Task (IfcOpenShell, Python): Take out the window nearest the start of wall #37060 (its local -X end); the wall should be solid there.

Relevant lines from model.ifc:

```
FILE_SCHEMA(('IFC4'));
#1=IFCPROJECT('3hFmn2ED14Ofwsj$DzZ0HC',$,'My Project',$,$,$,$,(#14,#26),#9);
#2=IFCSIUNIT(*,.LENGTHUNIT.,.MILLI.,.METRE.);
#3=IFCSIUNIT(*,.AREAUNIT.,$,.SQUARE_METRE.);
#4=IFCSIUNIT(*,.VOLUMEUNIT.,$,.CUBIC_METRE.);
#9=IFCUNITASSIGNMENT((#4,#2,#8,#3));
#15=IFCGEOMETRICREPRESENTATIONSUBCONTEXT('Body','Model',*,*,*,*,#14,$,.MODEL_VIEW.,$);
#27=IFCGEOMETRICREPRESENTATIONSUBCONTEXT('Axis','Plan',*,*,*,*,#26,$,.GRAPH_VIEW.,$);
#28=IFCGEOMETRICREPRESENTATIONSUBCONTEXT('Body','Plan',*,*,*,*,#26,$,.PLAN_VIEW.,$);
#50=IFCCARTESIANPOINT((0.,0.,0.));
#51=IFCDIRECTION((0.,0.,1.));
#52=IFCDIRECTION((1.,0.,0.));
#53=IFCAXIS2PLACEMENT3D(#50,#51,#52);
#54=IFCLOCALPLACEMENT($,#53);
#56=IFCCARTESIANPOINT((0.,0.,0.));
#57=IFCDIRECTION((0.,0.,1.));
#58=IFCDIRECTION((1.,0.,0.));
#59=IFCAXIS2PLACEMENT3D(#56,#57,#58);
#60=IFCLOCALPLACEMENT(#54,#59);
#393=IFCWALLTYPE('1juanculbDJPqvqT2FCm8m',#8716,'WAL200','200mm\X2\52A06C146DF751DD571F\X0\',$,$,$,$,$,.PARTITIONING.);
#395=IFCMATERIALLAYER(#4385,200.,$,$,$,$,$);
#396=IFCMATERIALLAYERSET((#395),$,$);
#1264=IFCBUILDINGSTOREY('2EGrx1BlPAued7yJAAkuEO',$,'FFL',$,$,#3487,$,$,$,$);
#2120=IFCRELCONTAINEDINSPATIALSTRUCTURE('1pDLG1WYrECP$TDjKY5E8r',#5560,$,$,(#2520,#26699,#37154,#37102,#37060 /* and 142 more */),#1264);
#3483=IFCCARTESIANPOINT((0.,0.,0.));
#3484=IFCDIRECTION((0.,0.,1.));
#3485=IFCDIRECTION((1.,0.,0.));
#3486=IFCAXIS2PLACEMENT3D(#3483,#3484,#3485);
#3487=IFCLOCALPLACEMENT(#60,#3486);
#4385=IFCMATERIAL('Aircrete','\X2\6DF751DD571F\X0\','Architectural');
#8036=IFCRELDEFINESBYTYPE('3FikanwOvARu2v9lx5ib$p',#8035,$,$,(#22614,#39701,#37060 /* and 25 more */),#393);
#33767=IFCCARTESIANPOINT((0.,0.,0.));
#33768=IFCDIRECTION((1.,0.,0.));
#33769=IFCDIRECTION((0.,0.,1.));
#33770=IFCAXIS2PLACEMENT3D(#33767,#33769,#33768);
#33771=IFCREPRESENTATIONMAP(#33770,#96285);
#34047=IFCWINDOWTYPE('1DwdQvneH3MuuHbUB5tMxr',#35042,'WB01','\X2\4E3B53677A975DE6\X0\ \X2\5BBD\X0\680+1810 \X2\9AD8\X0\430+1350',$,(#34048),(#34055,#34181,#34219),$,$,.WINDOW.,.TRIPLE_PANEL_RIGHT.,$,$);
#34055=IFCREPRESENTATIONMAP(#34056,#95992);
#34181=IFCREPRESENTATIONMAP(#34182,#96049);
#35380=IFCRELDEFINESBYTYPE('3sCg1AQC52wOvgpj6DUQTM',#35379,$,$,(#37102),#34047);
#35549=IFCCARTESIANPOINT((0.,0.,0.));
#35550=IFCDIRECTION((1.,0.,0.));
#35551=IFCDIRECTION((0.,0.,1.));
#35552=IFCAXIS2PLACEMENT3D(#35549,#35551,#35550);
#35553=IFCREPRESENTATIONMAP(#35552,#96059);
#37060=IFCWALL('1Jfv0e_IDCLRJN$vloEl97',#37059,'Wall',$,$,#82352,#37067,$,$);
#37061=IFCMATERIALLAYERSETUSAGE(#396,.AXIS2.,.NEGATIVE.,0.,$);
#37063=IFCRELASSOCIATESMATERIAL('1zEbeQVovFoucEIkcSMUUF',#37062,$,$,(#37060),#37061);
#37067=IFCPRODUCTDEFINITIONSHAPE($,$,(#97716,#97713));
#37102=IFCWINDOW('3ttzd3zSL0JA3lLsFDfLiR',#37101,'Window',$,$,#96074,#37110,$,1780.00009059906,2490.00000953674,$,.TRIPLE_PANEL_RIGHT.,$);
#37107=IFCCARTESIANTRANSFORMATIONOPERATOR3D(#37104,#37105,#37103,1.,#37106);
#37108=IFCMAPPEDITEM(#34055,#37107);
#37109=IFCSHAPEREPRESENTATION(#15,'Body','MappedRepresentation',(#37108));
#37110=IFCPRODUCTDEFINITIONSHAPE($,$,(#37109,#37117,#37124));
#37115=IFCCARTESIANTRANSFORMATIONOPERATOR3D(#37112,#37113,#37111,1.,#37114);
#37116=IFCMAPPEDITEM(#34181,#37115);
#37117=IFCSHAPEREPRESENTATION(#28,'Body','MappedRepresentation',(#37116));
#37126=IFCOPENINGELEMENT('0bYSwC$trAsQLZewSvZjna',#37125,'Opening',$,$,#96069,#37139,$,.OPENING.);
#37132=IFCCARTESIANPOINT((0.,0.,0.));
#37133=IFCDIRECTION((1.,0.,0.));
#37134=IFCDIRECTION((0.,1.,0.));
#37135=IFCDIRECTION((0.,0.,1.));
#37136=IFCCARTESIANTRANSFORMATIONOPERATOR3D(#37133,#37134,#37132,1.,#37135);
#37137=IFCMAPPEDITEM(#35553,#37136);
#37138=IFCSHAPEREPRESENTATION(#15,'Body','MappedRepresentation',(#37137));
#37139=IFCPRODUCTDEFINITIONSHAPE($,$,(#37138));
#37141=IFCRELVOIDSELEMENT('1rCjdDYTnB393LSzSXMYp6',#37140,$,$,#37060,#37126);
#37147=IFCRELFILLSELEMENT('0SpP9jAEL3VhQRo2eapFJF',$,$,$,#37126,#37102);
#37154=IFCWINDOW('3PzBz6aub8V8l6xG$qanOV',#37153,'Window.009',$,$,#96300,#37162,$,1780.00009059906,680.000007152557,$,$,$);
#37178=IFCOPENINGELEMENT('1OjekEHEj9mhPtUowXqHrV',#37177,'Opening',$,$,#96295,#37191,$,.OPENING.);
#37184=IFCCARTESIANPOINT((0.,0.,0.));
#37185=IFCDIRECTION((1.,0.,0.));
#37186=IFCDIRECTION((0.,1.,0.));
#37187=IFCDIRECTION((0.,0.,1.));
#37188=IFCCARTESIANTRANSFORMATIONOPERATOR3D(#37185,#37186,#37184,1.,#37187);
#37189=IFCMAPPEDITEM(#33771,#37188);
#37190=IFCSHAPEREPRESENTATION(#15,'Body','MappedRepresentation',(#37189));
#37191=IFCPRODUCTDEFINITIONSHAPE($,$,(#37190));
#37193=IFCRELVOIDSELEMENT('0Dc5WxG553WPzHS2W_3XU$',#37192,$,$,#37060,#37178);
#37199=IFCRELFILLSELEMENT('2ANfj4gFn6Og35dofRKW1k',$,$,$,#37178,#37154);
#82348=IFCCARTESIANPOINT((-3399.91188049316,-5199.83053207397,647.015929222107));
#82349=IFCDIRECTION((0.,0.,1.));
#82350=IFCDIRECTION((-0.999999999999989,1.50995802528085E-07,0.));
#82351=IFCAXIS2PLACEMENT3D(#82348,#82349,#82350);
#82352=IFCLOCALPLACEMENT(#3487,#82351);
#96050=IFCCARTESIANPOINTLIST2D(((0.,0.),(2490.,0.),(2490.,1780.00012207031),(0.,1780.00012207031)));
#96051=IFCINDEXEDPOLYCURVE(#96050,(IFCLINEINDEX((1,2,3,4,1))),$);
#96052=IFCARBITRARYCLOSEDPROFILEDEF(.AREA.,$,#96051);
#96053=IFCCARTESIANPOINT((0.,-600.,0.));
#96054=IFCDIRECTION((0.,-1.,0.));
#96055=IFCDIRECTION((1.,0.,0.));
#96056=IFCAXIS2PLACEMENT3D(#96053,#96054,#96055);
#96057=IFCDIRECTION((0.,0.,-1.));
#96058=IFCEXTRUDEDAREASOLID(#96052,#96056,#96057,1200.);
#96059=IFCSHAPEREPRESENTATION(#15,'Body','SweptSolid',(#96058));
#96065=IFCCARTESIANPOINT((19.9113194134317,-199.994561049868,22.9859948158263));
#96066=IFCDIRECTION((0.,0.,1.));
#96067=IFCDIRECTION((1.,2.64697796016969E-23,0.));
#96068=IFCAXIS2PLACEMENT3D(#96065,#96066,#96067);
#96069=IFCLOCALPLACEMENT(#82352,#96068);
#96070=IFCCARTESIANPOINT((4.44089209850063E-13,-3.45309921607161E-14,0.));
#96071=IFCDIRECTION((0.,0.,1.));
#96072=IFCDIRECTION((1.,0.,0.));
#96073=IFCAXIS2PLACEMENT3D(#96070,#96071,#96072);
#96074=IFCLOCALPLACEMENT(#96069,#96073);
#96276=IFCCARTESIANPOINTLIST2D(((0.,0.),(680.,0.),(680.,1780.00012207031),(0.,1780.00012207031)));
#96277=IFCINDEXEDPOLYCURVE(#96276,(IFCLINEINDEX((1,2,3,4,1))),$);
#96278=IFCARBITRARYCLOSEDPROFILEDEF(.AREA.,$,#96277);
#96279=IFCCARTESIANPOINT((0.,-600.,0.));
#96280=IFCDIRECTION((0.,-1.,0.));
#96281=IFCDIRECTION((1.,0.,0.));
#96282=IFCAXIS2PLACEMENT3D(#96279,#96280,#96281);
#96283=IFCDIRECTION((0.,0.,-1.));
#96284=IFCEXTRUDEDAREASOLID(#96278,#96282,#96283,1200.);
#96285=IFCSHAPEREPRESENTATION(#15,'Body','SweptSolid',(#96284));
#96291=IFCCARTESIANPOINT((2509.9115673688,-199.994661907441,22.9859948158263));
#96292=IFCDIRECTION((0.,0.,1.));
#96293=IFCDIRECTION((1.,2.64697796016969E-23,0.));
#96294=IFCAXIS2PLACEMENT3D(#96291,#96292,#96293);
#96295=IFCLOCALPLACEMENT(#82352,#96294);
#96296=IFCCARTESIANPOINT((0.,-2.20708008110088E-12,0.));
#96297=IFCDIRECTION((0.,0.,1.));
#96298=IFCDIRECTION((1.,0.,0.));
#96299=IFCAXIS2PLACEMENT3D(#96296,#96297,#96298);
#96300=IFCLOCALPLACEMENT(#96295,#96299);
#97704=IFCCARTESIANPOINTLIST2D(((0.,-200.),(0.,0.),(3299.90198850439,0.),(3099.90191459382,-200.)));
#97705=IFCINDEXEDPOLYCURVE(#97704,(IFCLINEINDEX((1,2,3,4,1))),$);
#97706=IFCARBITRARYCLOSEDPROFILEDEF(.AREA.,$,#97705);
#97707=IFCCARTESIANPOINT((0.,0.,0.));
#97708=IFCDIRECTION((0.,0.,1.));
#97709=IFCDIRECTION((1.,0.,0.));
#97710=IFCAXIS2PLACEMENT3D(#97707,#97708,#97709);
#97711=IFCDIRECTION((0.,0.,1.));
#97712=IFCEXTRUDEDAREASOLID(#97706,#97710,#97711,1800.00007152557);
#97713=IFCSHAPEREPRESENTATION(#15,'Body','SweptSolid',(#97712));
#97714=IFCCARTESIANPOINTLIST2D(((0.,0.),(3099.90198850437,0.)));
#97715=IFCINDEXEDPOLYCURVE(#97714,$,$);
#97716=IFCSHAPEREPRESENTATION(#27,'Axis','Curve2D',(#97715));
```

```python
import ifcopenshell
import ifcopenshell.api.feature
import ifcopenshell.api.root
import ifcopenshell.geom
import ifcopenshell.util.shape

model = ifcopenshell.open("model.ifc")
settings = ifcopenshell.geom.settings()


def volume(element):
    """Net volume in cubic metres, openings subtracted."""
    shape = ifcopenshell.geom.create_shape(settings, element)
    return ifcopenshell.util.shape.get_volume(shape.geometry)


window = model.by_id(37102)
opening = window.FillsVoids[0].RelatingOpeningElement
wall = opening.VoidsElements[0].RelatingBuildingElement
before = volume(wall)

ifcopenshell.api.root.remove_product(model, product=window)
ifcopenshell.api.feature.remove_feature(model, feature=opening)

after = volume(wall)

print(f"wall volume {before:.3f} -> {after:.3f} m3")

model.write("model-out.ifc")
```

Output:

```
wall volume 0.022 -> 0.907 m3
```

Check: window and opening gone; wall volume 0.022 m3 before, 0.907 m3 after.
